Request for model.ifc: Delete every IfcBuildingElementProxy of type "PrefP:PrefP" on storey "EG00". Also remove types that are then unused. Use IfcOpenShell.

First a look at what the model holds.

```python
import ifcopenshell
import ifcopenshell.util.element

model = ifcopenshell.open("model.ifc")
print(model.schema)
storey = next(s for s in model.by_type("IfcBuildingStorey") if s.Name == "EG00")
proxies = [e for e in ifcopenshell.util.element.get_decomposition(storey) if e.is_a("IfcBuildingElementProxy")]
seen = {}
for e in proxies:
    element_type = ifcopenshell.util.element.get_type(e)
    name = element_type.Name if element_type not in (None, e) else None
    seen[name] = seen.get(name, 0) + 1
for name, count in sorted(seen.items(), key=str):
    print(count, "x", name)
```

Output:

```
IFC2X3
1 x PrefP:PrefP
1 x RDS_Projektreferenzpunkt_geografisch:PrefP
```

```python
import ifcopenshell
import ifcopenshell.api.root
import ifcopenshell.util.element

model = ifcopenshell.open("model.ifc")

storey = next(s for s in model.by_type("IfcBuildingStorey") if s.Name == "EG00")
proxies = [e for e in ifcopenshell.util.element.get_decomposition(storey) if e.is_a("IfcBuildingElementProxy")]
targets = [e for e in proxies if (t := ifcopenshell.util.element.get_type(e)) not in (None, e) and t.Name == "PrefP:PrefP"]
types = {ifcopenshell.util.element.get_type(e) for e in targets} - {None, *targets}

for e in targets:
    ifcopenshell.api.root.remove_product(model, product=e)
print(len(targets), "removed")

unused = [t for t in types if not ifcopenshell.util.element.get_types(t)]
for t in unused:
    ifcopenshell.api.root.remove_product(model, product=t)
print(len(unused), "unused types removed")

model.write("model_rev.ifc")
```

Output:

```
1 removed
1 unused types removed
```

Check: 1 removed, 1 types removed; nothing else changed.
